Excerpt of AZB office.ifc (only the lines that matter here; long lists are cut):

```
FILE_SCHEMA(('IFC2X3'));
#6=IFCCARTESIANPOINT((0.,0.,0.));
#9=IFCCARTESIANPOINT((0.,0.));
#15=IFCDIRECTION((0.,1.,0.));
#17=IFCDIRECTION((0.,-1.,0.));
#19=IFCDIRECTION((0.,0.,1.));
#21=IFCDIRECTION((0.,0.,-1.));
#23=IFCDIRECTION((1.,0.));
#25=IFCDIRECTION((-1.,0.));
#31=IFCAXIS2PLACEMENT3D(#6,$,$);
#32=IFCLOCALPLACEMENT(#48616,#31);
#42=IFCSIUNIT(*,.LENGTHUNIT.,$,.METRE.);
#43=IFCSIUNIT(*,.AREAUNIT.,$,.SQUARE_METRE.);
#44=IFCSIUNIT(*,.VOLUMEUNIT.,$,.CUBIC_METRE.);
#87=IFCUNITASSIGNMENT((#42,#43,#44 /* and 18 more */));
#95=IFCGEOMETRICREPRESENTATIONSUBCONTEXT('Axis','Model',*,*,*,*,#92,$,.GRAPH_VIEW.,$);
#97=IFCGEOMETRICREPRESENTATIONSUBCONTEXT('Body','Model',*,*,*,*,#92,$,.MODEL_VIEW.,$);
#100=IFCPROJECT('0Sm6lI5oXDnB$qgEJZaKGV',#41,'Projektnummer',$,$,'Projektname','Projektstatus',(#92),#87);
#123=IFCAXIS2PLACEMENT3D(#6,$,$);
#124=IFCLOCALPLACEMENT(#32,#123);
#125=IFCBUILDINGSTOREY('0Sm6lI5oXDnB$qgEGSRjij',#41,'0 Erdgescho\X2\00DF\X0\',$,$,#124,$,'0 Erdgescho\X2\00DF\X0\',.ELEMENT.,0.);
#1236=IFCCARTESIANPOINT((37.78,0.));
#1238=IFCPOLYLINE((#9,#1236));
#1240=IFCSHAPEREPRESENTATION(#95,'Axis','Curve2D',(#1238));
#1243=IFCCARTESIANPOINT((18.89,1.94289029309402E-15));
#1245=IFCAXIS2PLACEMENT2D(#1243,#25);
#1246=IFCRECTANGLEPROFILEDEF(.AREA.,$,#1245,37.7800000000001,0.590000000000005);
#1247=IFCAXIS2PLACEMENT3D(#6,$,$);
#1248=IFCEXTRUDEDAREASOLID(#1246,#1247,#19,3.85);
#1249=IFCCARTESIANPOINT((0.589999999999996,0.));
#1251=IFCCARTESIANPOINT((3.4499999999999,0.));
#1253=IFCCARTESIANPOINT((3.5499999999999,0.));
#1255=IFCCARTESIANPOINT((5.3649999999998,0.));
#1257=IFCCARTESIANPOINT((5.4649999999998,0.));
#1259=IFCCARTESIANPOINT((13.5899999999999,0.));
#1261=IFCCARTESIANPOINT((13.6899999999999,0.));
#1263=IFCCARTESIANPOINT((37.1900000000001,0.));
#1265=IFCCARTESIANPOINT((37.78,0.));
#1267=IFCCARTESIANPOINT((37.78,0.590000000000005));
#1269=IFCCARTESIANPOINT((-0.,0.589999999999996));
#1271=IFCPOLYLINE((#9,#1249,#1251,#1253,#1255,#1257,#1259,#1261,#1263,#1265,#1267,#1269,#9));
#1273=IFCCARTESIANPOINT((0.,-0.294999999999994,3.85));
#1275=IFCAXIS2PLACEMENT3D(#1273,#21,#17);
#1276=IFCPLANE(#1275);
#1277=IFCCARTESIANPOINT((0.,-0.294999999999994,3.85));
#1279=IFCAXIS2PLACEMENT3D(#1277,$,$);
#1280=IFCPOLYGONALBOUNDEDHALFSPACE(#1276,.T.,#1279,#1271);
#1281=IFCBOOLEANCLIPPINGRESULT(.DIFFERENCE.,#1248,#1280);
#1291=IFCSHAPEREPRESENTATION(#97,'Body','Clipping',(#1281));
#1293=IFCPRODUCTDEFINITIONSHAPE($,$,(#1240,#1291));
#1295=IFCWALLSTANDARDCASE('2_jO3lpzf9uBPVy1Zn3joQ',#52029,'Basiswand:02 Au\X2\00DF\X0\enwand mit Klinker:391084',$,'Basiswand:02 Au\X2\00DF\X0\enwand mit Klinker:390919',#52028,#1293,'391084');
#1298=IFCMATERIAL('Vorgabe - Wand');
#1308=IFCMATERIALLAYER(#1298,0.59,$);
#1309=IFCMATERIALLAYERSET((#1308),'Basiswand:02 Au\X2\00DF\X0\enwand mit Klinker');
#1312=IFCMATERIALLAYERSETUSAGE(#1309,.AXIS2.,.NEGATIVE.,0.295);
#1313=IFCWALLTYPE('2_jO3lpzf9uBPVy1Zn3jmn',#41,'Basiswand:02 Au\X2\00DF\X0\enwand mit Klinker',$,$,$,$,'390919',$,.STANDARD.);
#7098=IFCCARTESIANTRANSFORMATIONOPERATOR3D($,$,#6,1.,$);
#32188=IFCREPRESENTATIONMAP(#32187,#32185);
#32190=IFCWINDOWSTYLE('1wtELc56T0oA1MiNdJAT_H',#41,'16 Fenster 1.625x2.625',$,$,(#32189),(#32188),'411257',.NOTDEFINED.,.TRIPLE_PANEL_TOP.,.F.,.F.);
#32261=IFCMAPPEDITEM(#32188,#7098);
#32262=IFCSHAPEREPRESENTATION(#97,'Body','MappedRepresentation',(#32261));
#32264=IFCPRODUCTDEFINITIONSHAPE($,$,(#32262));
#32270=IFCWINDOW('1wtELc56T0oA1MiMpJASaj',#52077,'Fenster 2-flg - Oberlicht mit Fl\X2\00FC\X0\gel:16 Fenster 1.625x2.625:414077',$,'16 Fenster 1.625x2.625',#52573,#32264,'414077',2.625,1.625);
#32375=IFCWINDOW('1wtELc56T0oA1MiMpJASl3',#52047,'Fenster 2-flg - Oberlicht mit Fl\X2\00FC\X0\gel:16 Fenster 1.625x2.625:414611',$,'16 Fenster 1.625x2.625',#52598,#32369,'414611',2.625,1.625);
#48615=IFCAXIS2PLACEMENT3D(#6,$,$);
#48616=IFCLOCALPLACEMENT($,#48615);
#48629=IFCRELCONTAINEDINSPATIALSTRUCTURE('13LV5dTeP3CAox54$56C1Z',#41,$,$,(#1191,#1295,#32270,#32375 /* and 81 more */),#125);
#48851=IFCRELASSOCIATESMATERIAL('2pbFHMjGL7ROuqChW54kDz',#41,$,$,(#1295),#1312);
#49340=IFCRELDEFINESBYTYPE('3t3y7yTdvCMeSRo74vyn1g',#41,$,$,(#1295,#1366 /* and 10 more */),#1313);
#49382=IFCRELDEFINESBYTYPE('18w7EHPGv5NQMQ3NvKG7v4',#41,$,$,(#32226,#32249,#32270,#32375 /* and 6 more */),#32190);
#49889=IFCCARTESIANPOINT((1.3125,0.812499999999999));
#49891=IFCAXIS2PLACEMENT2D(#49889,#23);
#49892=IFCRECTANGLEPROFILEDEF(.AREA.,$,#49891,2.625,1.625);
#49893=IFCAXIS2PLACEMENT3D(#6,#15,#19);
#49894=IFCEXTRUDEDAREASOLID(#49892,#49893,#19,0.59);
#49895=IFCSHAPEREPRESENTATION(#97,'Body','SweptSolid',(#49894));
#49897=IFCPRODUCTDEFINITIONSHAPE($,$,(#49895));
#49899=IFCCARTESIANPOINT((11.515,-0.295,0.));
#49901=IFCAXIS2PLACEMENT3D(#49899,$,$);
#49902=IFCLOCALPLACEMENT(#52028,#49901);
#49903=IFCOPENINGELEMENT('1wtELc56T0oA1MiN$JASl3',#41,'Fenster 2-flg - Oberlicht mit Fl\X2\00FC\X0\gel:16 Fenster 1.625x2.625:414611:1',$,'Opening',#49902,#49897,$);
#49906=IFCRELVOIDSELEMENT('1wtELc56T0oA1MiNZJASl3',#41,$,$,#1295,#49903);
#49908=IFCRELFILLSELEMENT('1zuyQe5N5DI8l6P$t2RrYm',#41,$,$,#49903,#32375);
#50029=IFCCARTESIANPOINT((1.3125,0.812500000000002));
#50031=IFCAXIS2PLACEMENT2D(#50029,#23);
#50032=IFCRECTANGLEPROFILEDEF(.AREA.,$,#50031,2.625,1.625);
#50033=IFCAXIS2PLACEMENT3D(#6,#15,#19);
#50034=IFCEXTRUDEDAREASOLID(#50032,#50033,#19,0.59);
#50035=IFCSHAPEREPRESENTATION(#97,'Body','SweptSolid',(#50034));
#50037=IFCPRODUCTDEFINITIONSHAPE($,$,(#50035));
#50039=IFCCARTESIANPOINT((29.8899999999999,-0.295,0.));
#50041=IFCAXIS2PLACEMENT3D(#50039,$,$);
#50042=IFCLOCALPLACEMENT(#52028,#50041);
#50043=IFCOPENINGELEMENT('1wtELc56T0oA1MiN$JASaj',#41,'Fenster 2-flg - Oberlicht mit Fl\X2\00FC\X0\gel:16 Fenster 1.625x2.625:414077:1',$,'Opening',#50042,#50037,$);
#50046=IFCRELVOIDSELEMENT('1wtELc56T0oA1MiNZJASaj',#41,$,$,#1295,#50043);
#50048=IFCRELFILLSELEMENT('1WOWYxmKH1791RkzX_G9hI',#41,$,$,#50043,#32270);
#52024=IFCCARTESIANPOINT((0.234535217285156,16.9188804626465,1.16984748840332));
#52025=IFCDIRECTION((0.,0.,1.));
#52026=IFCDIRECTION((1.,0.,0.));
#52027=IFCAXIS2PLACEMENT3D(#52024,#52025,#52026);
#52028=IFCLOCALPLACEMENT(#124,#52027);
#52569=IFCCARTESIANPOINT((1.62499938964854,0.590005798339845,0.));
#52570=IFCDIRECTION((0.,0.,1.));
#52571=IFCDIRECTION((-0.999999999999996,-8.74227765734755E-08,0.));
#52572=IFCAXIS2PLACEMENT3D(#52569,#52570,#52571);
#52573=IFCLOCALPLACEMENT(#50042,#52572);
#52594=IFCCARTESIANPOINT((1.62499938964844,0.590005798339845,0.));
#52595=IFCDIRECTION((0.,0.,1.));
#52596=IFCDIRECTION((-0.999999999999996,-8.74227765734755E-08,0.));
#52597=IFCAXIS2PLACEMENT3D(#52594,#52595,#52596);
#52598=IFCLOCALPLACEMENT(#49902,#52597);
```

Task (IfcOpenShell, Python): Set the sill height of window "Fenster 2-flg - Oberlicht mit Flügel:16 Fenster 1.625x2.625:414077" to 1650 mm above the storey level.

```python
import numpy as np
import ifcopenshell
import ifcopenshell.api.geometry
import ifcopenshell.geom
import ifcopenshell.util.element
import ifcopenshell.util.placement
import ifcopenshell.util.shape
import ifcopenshell.util.unit

model = ifcopenshell.open("AZB office.ifc")
unit_scale = ifcopenshell.util.unit.calculate_unit_scale(model)

window = model.by_guid("1wtELc56T0oA1MiMpJASaj")
opening = window.FillsVoids[0].RelatingOpeningElement
storey = ifcopenshell.util.element.get_container(window, ifc_class="IfcBuildingStorey")
level = ifcopenshell.util.placement.get_local_placement(storey.ObjectPlacement)[2, 3]

# The opening's origin need not be at the sill, so measure its lowest point.
shape = ifcopenshell.geom.create_shape(ifcopenshell.geom.settings(), opening)
bottom = ifcopenshell.util.shape.get_shape_bottom_elevation(shape, shape.geometry) / unit_scale
dz = level + 1.65 - bottom

shift = np.array([0.0, 0.0, dz])
# The window is placed relative to its opening, so it follows when the opening moves.
matrix = ifcopenshell.util.placement.get_local_placement(opening.ObjectPlacement)
matrix[:3, 3] += shift
ifcopenshell.api.geometry.edit_object_placement(
    model, product=opening, matrix=matrix, is_si=False, should_transform_children=True
)

print(f"moved by {dz * unit_scale:+.3f} m")

model.write("AZB office_edited.ifc")
```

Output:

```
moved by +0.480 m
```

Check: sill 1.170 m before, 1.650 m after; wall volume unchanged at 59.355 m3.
